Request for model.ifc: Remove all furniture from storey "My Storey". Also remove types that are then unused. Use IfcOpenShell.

First a look at what the model holds.

```python
import ifcopenshell
import ifcopenshell.util.element

model = ifcopenshell.open("model.ifc")
print(model.schema)
storey = next(s for s in model.by_type("IfcBuildingStorey") if s.Name == "My Storey")
furniture = [e for e in ifcopenshell.util.element.get_decomposition(storey) if e.is_a("IfcFurnishingElement")]
seen = {}
for e in furniture:
    element_type = ifcopenshell.util.element.get_type(e)
    name = element_type.Name if element_type not in (None, e) else None
    seen[name] = seen.get(name, 0) + 1
for name, count in sorted(seen.items(), key=str):
    print(count, "x", name)
```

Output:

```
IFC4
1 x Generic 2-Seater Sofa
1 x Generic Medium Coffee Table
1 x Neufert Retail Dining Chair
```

```python
import ifcopenshell
import ifcopenshell.api.root
import ifcopenshell.util.element

model = ifcopenshell.open("model.ifc")

storey = next(s for s in model.by_type("IfcBuildingStorey") if s.Name == "My Storey")
furniture = [e for e in ifcopenshell.util.element.get_decomposition(storey) if e.is_a("IfcFurnishingElement")]
types = {ifcopenshell.util.element.get_type(e) for e in furniture} - {None, *furniture}

for e in furniture:
    ifcopenshell.api.root.remove_product(model, product=e)
print(len(furniture), "removed")

unused = [t for t in types if not ifcopenshell.util.element.get_types(t)]
for t in unused:
    ifcopenshell.api.root.remove_product(model, product=t)
print(len(unused), "unused types removed")

model.write("model-out.ifc")
```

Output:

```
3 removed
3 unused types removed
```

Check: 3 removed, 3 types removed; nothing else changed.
